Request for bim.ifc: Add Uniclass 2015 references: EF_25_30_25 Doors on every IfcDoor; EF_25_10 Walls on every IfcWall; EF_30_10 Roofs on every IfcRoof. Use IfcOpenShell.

First a look at what the model holds.

```python
import ifcopenshell

model = ifcopenshell.open("bim.ifc")
print(model.schema)
print("classifications:", [c.Name for c in model.by_type("IfcClassification")])
for ifc_class in ("IfcDoor", "IfcRoof", "IfcStair", "IfcWall", "IfcWindow"):
    print(ifc_class, len(model.by_type(ifc_class)))
```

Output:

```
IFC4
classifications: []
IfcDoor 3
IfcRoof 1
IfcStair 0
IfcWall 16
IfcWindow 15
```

```python
import ifcopenshell
import ifcopenshell.api.classification

model = ifcopenshell.open("bim.ifc")

system = ifcopenshell.api.classification.add_classification(model, classification="Uniclass 2015")

codes = {
    "IfcDoor": ("EF_25_30_25", "Doors"),
    "IfcWall": ("EF_25_10", "Walls"),
    "IfcRoof": ("EF_30_10", "Roofs"),
}
for ifc_class, (code, name) in codes.items():
    products = model.by_type(ifc_class)
    ifcopenshell.api.classification.add_reference(
        model, products=products, classification=system, identification=code, name=name
    )
    print(code, len(products))

model.write("bim_rev.ifc")
```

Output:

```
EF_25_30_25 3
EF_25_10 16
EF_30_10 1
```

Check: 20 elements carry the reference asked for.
